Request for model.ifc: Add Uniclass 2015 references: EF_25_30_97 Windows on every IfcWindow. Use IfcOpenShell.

First a look at what the model holds.

```python
import ifcopenshell

model = ifcopenshell.open("model.ifc")
print(model.schema)
print("classifications:", [c.Name for c in model.by_type("IfcClassification")])
for ifc_class in ("IfcDoor", "IfcRoof", "IfcStair", "IfcWall", "IfcWindow"):
    print(ifc_class, len(model.by_type(ifc_class)))
```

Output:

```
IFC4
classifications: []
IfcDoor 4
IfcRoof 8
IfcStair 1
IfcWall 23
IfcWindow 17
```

```python
import ifcopenshell
import ifcopenshell.api.classification

model = ifcopenshell.open("model.ifc")

system = ifcopenshell.api.classification.add_classification(model, classification="Uniclass 2015")

codes = {
    "IfcWindow": ("EF_25_30_97", "Windows"),
}
for ifc_class, (code, name) in codes.items():
    products = model.by_type(ifc_class)
    ifcopenshell.api.classification.add_reference(
        model, products=products, classification=system, identification=code, name=name
    )
    print(code, len(products))

model.write("model_v2.ifc")
```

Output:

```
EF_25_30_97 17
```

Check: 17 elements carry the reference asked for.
